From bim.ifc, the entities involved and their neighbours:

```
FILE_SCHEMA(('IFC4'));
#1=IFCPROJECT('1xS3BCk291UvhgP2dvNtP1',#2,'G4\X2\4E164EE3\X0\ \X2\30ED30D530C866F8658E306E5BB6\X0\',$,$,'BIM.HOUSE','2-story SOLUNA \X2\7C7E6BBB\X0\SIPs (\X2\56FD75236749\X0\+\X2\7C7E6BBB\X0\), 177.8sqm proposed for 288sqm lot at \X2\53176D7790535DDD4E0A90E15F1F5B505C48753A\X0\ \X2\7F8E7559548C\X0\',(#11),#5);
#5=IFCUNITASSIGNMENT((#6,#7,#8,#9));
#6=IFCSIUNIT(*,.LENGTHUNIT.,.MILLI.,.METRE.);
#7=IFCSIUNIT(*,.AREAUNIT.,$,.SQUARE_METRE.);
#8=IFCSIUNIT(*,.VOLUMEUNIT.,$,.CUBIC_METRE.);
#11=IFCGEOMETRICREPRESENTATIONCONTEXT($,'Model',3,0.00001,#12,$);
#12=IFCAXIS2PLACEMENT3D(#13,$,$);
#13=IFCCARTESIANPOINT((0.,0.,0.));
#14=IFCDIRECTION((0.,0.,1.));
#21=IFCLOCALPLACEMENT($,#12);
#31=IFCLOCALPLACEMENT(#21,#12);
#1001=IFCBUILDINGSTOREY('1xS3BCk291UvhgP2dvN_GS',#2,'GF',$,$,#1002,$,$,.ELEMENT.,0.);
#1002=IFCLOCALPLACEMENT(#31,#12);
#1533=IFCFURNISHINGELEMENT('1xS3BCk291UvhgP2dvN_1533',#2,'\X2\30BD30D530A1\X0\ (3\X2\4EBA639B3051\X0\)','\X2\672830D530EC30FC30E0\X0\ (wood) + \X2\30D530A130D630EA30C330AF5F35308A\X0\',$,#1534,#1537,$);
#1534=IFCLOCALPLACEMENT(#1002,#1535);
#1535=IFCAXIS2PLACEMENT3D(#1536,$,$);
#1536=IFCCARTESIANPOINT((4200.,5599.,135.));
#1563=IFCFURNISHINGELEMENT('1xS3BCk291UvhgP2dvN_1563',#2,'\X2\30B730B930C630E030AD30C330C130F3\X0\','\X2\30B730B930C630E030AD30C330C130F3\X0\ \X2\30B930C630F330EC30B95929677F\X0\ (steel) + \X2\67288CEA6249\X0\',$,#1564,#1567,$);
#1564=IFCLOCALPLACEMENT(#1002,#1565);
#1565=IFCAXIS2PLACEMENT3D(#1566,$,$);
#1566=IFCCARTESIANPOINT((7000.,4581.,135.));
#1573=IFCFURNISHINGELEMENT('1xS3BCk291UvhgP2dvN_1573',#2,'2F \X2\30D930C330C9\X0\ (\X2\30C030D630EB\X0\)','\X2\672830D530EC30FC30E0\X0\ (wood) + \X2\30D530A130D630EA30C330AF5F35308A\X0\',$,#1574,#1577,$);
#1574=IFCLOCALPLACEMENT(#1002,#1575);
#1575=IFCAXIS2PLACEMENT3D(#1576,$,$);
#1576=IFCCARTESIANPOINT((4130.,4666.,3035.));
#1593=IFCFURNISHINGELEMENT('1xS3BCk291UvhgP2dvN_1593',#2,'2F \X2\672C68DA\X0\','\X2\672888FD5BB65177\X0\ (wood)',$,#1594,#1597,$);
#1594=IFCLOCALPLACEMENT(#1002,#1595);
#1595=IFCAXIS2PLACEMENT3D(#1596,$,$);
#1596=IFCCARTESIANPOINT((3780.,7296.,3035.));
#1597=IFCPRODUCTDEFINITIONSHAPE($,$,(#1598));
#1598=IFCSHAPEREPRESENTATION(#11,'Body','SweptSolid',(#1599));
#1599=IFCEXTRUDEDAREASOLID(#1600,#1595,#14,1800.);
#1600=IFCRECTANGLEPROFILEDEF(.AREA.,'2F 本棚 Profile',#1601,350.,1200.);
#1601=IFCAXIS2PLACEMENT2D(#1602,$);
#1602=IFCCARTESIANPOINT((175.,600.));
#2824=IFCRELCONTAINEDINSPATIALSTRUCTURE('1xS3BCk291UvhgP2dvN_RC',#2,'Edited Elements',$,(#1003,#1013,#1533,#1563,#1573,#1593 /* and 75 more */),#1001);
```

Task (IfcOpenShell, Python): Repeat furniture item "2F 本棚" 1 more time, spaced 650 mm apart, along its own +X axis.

```python
import ifcopenshell
import ifcopenshell.api.geometry
import ifcopenshell.api.root
import ifcopenshell.util.element
import ifcopenshell.util.placement
import ifcopenshell.util.unit

model = ifcopenshell.open("bim.ifc")
unit_scale = ifcopenshell.util.unit.calculate_unit_scale(model)


def reuse_history(source, copy):
    """copy_class also copies each property set's owner history, people and application; keep the originals."""
    for rel in copy.IsDefinedBy:
        if rel.is_a("IfcRelDefinesByProperties") and (history := rel.RelatingPropertyDefinition.OwnerHistory):
            rel.RelatingPropertyDefinition.OwnerHistory = source.OwnerHistory
            ifcopenshell.util.element.remove_deep2(model, history)


source = model.by_id(1593)
base = ifcopenshell.util.placement.get_local_placement(source.ObjectPlacement)
step = base[:3, 0] * 0.65 / unit_scale

for i in range(1, 2):
    copy = ifcopenshell.api.root.copy_class(model, product=source)
    copy.Representation = ifcopenshell.util.element.copy_deep(
        model, source.Representation, exclude=["IfcGeometricRepresentationContext", "IfcRepresentationMap"]
    )
    reuse_history(source, copy)
    matrix = base.copy()
    matrix[:3, 3] += i * step
    print("added at", matrix[:3, 3].round(3) + 0.0)
    ifcopenshell.api.geometry.edit_object_placement(model, product=copy, matrix=matrix, is_si=False)

model.write("bim_rev.ifc")
```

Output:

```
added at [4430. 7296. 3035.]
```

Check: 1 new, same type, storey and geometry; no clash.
